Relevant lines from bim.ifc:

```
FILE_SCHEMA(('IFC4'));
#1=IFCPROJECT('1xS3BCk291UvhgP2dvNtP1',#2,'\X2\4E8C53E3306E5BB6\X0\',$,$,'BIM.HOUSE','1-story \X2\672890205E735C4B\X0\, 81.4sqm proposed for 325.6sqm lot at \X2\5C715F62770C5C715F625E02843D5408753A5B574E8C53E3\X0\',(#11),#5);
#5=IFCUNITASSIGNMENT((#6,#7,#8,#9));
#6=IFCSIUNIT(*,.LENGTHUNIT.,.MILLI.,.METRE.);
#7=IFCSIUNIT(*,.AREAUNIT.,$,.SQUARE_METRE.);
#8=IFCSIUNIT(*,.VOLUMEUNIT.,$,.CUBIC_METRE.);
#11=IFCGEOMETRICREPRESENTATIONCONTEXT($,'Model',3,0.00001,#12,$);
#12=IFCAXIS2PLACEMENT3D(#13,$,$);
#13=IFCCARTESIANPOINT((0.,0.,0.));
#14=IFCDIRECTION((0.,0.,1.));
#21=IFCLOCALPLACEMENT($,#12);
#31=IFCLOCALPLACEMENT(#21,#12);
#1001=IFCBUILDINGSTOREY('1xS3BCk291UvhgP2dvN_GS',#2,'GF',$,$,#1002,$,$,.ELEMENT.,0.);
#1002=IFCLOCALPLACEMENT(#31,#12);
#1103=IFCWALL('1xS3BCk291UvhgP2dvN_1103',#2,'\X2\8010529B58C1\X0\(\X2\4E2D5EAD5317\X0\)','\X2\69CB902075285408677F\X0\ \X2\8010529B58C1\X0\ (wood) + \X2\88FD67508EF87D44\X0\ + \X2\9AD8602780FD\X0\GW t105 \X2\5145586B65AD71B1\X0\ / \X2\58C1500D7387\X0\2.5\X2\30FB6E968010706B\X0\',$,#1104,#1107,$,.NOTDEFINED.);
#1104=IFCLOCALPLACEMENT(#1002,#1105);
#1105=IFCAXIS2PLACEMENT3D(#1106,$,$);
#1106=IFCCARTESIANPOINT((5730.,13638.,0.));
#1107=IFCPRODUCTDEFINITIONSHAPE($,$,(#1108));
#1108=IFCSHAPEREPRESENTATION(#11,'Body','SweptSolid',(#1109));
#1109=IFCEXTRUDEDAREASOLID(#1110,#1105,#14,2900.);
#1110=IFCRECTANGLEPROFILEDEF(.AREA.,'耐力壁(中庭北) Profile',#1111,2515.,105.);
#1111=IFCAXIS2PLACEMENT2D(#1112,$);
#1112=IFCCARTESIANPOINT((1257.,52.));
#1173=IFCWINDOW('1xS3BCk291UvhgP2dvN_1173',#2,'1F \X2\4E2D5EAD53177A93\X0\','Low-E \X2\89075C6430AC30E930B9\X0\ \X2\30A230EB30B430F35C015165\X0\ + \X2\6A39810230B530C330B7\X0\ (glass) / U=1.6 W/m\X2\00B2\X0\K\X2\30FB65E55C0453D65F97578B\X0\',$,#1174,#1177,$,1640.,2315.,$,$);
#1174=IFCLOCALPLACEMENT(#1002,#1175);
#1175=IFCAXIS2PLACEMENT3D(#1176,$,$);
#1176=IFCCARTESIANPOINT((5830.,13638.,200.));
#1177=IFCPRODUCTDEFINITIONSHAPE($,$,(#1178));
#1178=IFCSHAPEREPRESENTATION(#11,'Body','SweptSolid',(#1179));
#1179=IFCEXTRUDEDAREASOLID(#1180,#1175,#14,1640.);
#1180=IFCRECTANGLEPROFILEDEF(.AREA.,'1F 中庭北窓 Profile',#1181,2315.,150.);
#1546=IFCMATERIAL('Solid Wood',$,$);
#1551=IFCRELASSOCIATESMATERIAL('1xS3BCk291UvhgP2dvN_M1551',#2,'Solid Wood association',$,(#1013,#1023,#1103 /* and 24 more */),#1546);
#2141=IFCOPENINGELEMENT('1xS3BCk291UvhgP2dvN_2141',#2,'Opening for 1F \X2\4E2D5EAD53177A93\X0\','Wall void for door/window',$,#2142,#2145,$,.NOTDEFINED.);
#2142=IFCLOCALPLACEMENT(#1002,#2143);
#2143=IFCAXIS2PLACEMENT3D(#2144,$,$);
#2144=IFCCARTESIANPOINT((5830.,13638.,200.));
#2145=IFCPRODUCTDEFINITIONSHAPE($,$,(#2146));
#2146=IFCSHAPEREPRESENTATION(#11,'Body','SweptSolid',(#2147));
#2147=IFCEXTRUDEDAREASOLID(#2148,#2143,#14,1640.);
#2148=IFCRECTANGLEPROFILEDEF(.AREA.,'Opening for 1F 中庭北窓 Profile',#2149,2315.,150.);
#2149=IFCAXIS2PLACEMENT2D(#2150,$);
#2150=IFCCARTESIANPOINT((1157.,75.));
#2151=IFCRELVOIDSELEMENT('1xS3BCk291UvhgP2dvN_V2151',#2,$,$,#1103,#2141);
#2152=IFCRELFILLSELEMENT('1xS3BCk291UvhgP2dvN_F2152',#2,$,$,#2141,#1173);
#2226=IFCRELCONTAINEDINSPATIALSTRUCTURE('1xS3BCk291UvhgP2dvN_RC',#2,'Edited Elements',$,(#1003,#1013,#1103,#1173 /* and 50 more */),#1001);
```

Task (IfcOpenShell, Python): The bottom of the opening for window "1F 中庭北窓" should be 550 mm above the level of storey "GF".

```python
import numpy as np
import ifcopenshell
import ifcopenshell.api.geometry
import ifcopenshell.geom
import ifcopenshell.util.element
import ifcopenshell.util.placement
import ifcopenshell.util.shape
import ifcopenshell.util.unit

model = ifcopenshell.open("bim.ifc")
unit_scale = ifcopenshell.util.unit.calculate_unit_scale(model)

window = model.by_guid("1xS3BCk291UvhgP2dvN_1173")
opening = window.FillsVoids[0].RelatingOpeningElement
storey = ifcopenshell.util.element.get_container(window, ifc_class="IfcBuildingStorey")
level = ifcopenshell.util.placement.get_local_placement(storey.ObjectPlacement)[2, 3]

# The opening's origin need not be at the sill, so measure its lowest point.
shape = ifcopenshell.geom.create_shape(ifcopenshell.geom.settings(), opening)
bottom = ifcopenshell.util.shape.get_shape_bottom_elevation(shape, shape.geometry) / unit_scale
dz = level + 550.0 - bottom

shift = np.array([0.0, 0.0, dz])
# The window is not placed relative to its opening, so move both.
for product in (opening, window):
    matrix = ifcopenshell.util.placement.get_local_placement(product.ObjectPlacement)
    matrix[:3, 3] += shift
    ifcopenshell.api.geometry.edit_object_placement(model, product=product, matrix=matrix, is_si=False)

print(f"moved by {dz * unit_scale:+.3f} m")

model.write("bim_updated.ifc")
```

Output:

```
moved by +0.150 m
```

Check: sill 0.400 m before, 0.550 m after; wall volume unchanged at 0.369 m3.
